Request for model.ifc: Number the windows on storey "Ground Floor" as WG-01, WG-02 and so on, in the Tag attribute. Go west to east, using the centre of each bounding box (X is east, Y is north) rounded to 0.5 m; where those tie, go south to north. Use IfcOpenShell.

First a look at what the model holds.

```python
import ifcopenshell
import ifcopenshell.util.element
import ifcopenshell.util.placement

model = ifcopenshell.open("model.ifc")
print(model.schema)
storey = next(s for s in model.by_type("IfcBuildingStorey") if s.Name == "Ground Floor")
windows = [e for e in ifcopenshell.util.element.get_decomposition(storey) if e.is_a("IfcWindow")]
for e in sorted(windows, key=lambda e: e.id()):
    origin = ifcopenshell.util.placement.get_local_placement(e.ObjectPlacement)[:3, 3]
    print(e.id(), e.Tag, e.Name, origin.round(2) + 0.0, sep=" | ")
```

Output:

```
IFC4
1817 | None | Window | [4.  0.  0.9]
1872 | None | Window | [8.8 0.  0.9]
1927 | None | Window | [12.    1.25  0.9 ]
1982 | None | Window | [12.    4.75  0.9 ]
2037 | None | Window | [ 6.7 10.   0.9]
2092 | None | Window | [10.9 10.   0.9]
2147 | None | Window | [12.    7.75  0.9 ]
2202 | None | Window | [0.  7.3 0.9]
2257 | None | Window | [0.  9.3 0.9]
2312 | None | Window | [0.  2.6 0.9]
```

```python
import ifcopenshell
import ifcopenshell.geom
import ifcopenshell.util.element
import ifcopenshell.util.shape

model = ifcopenshell.open("model.ifc")
settings = ifcopenshell.geom.settings()
settings.set("use-world-coords", True)


def centre(element):
    shape = ifcopenshell.geom.create_shape(settings, element)
    return ifcopenshell.util.shape.get_bbox_centroid(shape.geometry)


storey = next(s for s in model.by_type("IfcBuildingStorey") if s.Name == "Ground Floor")
windows = [e for e in ifcopenshell.util.element.get_decomposition(storey) if e.is_a("IfcWindow")]

# Insertion points can sit at a corner or the storey origin, so sort by the geometry (in metres).
centres = {e: centre(e) for e in windows}
windows.sort(key=lambda e: (round(centres[e][0] / 0.5), centres[e][1]))

for i, e in enumerate(windows, start=1):
    number = f"WG-{i:02d}"
    e.Tag = number
    print(e.id(), number)

model.write("model_v2.ifc")
```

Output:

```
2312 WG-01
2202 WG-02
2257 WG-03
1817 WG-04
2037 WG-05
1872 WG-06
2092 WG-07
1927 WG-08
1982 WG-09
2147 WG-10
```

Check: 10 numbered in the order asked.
